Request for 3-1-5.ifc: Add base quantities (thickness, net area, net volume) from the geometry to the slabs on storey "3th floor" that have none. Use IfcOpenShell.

First a look at what the model holds.

```python
import ifcopenshell
import ifcopenshell.util.element
import ifcopenshell.util.unit

model = ifcopenshell.open("3-1-5.ifc")
print(model.schema)
for unit_type in ("LENGTHUNIT", "AREAUNIT", "VOLUMEUNIT"):
    print(unit_type, ifcopenshell.util.unit.calculate_unit_scale(model, unit_type))
storey = next(s for s in model.by_type("IfcBuildingStorey") if s.Name == "3th floor")
slabs = [e for e in ifcopenshell.util.element.get_decomposition(storey) if e.is_a("IfcSlab")]
for e in sorted(slabs, key=lambda e: e.id()):
    print(e.id(), e.is_a(), e.Name, list(ifcopenshell.util.element.get_psets(e, qtos_only=True)), sep=" | ")
```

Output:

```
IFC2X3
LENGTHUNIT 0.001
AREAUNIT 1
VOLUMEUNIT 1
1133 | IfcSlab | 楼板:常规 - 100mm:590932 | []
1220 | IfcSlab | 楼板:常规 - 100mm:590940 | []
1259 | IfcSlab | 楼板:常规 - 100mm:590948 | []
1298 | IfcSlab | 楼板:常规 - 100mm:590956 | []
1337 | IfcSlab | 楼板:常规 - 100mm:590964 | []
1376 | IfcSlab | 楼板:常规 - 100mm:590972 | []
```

```python
import ifcopenshell
import ifcopenshell.api.pset
import ifcopenshell.geom
import ifcopenshell.util.element
import ifcopenshell.util.shape
import ifcopenshell.util.unit

model = ifcopenshell.open("3-1-5.ifc")
unit_scale = ifcopenshell.util.unit.calculate_unit_scale(model)
area_scale = ifcopenshell.util.unit.calculate_unit_scale(model, "AREAUNIT")
volume_scale = ifcopenshell.util.unit.calculate_unit_scale(model, "VOLUMEUNIT")
settings = ifcopenshell.geom.settings()

storey = next(s for s in model.by_type("IfcBuildingStorey") if s.Name == "3th floor")
slabs = [e for e in ifcopenshell.util.element.get_decomposition(storey) if e.is_a("IfcSlab")]

for e in sorted(slabs, key=lambda e: e.id()):
    if ifcopenshell.util.element.get_psets(e, qtos_only=True, should_inherit=False):
        continue
    # Geometry comes back in metres, in the element's own axes.
    shape = ifcopenshell.geom.create_shape(settings, e)
    values = {
        "Width": ifcopenshell.util.shape.get_z(shape.geometry) / unit_scale,
        "NetArea": ifcopenshell.util.shape.get_footprint_area(shape.geometry) / area_scale,
        "NetVolume": ifcopenshell.util.shape.get_volume(shape.geometry) / volume_scale,
    }
    qto = ifcopenshell.api.pset.add_qto(model, product=e, name="BaseQuantities")
    ifcopenshell.api.pset.edit_qto(model, qto=qto, properties=values)
    print(e.id(), {k: round(v, 3) for k, v in values.items()})

model.write("3-1-5_updated.ifc")
```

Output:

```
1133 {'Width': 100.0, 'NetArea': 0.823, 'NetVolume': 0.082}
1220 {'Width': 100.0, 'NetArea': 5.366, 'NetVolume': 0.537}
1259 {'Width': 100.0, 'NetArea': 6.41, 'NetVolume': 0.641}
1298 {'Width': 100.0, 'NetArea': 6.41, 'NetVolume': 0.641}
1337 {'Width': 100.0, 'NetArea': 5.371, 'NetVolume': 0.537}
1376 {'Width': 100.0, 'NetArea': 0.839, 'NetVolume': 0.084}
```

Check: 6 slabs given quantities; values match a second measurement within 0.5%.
